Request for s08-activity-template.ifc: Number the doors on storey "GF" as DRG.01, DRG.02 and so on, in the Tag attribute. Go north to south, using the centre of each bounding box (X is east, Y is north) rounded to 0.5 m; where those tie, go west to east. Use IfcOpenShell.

First a look at what the model holds.

```python
import ifcopenshell
import ifcopenshell.util.element
import ifcopenshell.util.placement

model = ifcopenshell.open("s08-activity-template.ifc")
print(model.schema)
storey = next(s for s in model.by_type("IfcBuildingStorey") if s.Name == "GF")
doors = [e for e in ifcopenshell.util.element.get_decomposition(storey) if e.is_a("IfcDoor")]
for e in sorted(doors, key=lambda e: e.id()):
    origin = ifcopenshell.util.placement.get_local_placement(e.ObjectPlacement)[:3, 3]
    print(e.id(), e.Tag, e.Name, origin.round(2) + 0.0, sep=" | ")
```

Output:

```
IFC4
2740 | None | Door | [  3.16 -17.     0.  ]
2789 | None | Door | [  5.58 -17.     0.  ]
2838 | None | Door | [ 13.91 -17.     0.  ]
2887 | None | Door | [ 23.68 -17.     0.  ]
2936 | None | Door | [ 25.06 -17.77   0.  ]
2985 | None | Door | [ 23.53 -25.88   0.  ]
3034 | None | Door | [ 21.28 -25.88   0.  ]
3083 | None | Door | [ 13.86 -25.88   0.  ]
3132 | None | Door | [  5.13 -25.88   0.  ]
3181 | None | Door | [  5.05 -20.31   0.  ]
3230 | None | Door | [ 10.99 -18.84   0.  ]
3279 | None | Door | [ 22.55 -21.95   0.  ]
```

```python
import ifcopenshell
import ifcopenshell.geom
import ifcopenshell.util.element
import ifcopenshell.util.shape

model = ifcopenshell.open("s08-activity-template.ifc")
settings = ifcopenshell.geom.settings()
settings.set("use-world-coords", True)


def centre(element):
    shape = ifcopenshell.geom.create_shape(settings, element)
    return ifcopenshell.util.shape.get_bbox_centroid(shape.geometry)


storey = next(s for s in model.by_type("IfcBuildingStorey") if s.Name == "GF")
doors = [e for e in ifcopenshell.util.element.get_decomposition(storey) if e.is_a("IfcDoor")]

# Insertion points can sit at a corner or the storey origin, so sort by the geometry (in metres).
centres = {e: centre(e) for e in doors}
doors.sort(key=lambda e: (-round(centres[e][1] / 0.5), centres[e][0]))

for i, e in enumerate(doors, start=1):
    number = f"DRG.{i:02d}"
    e.Tag = number
    print(e.id(), number)

model.write("s08-activity-template-out.ifc")
```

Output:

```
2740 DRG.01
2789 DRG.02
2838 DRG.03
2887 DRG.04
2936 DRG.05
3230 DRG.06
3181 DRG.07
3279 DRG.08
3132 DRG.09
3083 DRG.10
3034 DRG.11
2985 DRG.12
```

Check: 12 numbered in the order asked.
